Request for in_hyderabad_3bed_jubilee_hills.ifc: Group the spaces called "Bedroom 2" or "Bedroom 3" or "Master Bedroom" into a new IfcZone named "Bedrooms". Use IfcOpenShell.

First a look at what the model holds.

```python
import ifcopenshell

model = ifcopenshell.open("in_hyderabad_3bed_jubilee_hills.ifc")
print(model.schema)
seen = {}
for space in model.by_type("IfcSpace"):
    seen[space.LongName] = seen.get(space.LongName, 0) + 1
for name, count in sorted(seen.items(), key=str):
    print(count, "x", name)
print("zones:", [z.Name for z in model.by_type("IfcZone")][:20])
```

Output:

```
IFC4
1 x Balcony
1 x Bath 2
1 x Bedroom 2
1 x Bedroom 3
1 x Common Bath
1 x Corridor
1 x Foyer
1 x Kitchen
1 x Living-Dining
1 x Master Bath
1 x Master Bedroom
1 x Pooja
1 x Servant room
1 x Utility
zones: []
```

```python
import ifcopenshell
import ifcopenshell.api.group
import ifcopenshell.api.root

model = ifcopenshell.open("in_hyderabad_3bed_jubilee_hills.ifc")

names = {"Bedroom 2", "Bedroom 3", "Master Bedroom"}
spaces = [s for s in model.by_type("IfcSpace") if s.LongName in names]

zone = ifcopenshell.api.root.create_entity(model, ifc_class="IfcZone", name="Bedrooms")
ifcopenshell.api.group.assign_group(model, products=spaces, group=zone)
print(len(spaces), "spaces in", zone.Name)

model.write("in_hyderabad_3bed_jubilee_hills_v2.ifc")
```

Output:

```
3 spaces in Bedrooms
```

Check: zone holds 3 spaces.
